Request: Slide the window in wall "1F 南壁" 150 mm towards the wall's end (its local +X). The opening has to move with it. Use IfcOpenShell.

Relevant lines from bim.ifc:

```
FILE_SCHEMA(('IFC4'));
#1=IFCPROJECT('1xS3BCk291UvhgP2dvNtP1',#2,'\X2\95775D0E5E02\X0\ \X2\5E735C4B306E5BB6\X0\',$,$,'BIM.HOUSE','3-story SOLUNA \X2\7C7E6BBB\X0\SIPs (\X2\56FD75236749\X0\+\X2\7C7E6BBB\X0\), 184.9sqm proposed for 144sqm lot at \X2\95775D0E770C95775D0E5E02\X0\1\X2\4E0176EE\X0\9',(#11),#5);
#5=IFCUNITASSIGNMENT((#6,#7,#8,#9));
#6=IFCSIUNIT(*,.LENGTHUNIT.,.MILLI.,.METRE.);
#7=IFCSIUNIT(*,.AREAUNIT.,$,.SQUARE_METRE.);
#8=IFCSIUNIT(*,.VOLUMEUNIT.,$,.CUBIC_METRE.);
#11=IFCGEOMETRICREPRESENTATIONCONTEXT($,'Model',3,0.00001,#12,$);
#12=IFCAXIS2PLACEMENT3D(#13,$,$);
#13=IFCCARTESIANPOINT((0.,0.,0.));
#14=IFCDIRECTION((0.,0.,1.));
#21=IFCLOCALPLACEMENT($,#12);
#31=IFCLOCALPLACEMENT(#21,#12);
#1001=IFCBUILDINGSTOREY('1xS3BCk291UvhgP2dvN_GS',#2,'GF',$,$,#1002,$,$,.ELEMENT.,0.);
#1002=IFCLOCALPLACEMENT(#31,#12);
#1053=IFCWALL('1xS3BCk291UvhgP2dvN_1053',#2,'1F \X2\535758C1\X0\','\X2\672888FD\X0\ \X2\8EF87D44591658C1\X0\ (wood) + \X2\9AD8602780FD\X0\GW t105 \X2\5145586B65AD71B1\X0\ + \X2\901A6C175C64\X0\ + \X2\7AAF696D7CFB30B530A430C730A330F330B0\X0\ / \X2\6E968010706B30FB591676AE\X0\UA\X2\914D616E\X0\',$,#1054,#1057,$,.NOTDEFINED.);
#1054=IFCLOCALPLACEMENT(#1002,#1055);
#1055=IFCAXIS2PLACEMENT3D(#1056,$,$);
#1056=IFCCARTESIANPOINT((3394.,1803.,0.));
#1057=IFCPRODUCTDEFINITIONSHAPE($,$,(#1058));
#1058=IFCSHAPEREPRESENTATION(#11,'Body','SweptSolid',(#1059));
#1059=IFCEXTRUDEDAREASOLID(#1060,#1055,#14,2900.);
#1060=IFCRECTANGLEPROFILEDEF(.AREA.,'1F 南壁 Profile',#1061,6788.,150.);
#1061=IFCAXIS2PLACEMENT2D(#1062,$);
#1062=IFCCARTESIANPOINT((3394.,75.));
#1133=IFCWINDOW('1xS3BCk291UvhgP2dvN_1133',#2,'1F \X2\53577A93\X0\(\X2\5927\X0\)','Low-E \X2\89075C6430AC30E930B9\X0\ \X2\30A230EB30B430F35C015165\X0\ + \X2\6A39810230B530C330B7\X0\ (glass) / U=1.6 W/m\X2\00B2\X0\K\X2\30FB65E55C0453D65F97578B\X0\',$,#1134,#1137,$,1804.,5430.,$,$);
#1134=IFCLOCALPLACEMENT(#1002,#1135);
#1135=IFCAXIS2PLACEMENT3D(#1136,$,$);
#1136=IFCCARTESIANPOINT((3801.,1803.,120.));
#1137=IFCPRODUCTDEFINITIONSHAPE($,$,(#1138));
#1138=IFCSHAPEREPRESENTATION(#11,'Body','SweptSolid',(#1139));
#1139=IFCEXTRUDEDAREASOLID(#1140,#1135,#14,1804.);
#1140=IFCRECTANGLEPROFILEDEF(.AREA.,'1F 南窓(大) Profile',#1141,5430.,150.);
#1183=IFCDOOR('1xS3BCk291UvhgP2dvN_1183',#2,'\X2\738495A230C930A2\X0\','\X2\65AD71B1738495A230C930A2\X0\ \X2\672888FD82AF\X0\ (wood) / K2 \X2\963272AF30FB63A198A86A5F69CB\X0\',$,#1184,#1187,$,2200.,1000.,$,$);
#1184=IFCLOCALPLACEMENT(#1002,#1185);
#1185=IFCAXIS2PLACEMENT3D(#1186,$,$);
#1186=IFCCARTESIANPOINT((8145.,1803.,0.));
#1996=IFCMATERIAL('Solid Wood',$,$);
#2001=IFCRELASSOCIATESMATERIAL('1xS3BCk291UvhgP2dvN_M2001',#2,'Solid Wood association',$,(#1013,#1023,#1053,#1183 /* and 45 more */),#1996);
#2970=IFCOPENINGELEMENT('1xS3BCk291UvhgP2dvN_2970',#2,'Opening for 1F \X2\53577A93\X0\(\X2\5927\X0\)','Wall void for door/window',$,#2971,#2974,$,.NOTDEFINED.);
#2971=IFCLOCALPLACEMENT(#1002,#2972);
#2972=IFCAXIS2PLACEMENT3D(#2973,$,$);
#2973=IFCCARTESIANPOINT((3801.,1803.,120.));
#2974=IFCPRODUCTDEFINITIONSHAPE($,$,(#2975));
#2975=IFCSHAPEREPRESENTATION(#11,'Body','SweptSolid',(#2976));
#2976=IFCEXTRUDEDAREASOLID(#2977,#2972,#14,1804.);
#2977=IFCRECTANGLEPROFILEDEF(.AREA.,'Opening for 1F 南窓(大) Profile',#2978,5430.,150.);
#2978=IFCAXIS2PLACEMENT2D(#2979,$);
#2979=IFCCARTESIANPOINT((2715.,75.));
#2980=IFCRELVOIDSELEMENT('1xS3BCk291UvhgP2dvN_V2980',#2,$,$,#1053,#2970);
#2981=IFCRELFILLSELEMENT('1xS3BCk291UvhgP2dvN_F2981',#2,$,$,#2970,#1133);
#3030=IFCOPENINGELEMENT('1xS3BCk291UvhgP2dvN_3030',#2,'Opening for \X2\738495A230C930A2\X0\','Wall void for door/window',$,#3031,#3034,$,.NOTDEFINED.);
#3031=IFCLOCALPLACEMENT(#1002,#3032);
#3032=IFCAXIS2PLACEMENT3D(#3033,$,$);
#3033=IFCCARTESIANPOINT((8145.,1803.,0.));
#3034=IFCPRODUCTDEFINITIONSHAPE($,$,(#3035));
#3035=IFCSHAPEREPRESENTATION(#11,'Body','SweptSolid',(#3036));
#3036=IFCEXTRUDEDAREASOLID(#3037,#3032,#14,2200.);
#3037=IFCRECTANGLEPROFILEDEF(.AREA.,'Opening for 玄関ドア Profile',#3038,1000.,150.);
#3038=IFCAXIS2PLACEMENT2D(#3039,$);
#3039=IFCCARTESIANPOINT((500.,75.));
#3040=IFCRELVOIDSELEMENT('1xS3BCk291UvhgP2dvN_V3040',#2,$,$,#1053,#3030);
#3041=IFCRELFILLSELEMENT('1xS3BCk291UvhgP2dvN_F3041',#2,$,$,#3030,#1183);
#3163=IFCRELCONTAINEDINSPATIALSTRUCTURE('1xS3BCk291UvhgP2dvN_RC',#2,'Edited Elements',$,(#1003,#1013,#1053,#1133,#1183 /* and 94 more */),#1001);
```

```python
import ifcopenshell
import ifcopenshell.api.geometry
import ifcopenshell.util.placement
import ifcopenshell.util.unit

model = ifcopenshell.open("bim.ifc")
unit_scale = ifcopenshell.util.unit.calculate_unit_scale(model)

window = model.by_id(1133)
opening = window.FillsVoids[0].RelatingOpeningElement
wall = opening.VoidsElements[0].RelatingBuildingElement

wall_matrix = ifcopenshell.util.placement.get_local_placement(wall.ObjectPlacement)
shift = wall_matrix[:3, 0] * 0.15 / unit_scale
before = ifcopenshell.util.placement.get_local_placement(window.ObjectPlacement)[:3, 3].copy()

# The window is not placed relative to its opening, so move both.
for product in (opening, window):
    matrix = ifcopenshell.util.placement.get_local_placement(product.ObjectPlacement)
    matrix[:3, 3] += shift
    ifcopenshell.api.geometry.edit_object_placement(model, product=product, matrix=matrix, is_si=False)

after = ifcopenshell.util.placement.get_local_placement(window.ObjectPlacement)[:3, 3]
print("window moved by", (after - before).round(3) + 0.0)

model.write("bim_edited.ifc")
```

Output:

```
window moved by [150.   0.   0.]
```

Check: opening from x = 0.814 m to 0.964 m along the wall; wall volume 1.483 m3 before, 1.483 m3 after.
